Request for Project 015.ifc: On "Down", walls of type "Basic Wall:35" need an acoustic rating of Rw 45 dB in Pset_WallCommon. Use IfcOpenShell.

First a look at what the model holds.

```python
import ifcopenshell
import ifcopenshell.util.element

model = ifcopenshell.open("Project 015.ifc")
print(model.schema)
storey = next(s for s in model.by_type("IfcBuildingStorey") if s.Name == "Down")
walls = [e for e in ifcopenshell.util.element.get_decomposition(storey) if e.is_a("IfcWall")]
seen = {}
for e in walls:
    element_type = ifcopenshell.util.element.get_type(e)
    key = (element_type.Name if element_type != e and element_type else None, ifcopenshell.util.element.get_pset(e, "Pset_WallCommon", "AcousticRating"))
    seen[key] = seen.get(key, 0) + 1
for (name, value), count in sorted(seen.items(), key=str):
    print(count, "x", name, "|", value)
```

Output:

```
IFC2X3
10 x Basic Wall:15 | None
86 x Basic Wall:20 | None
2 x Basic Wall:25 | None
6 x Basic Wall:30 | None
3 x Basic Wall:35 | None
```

```python
import ifcopenshell
import ifcopenshell.api.pset
import ifcopenshell.util.element

model = ifcopenshell.open("Project 015.ifc")

storey = next(s for s in model.by_type("IfcBuildingStorey") if s.Name == "Down")
walls = [e for e in ifcopenshell.util.element.get_decomposition(storey) if e.is_a("IfcWall")]

count = 0
for e in walls:
    element_type = ifcopenshell.util.element.get_type(e)
    if element_type in (None, e) or element_type.Name != "Basic Wall:35":
        continue
    # add_pset returns the element's existing set when there is one.
    pset = ifcopenshell.api.pset.add_pset(model, product=e, name="Pset_WallCommon")
    ifcopenshell.api.pset.edit_pset(model, pset=pset, properties={"AcousticRating": "Rw 45 dB"})
    count += 1

print(count, "walls updated")

model.write("Project 015_v2.ifc")
```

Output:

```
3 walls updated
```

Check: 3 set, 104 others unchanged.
